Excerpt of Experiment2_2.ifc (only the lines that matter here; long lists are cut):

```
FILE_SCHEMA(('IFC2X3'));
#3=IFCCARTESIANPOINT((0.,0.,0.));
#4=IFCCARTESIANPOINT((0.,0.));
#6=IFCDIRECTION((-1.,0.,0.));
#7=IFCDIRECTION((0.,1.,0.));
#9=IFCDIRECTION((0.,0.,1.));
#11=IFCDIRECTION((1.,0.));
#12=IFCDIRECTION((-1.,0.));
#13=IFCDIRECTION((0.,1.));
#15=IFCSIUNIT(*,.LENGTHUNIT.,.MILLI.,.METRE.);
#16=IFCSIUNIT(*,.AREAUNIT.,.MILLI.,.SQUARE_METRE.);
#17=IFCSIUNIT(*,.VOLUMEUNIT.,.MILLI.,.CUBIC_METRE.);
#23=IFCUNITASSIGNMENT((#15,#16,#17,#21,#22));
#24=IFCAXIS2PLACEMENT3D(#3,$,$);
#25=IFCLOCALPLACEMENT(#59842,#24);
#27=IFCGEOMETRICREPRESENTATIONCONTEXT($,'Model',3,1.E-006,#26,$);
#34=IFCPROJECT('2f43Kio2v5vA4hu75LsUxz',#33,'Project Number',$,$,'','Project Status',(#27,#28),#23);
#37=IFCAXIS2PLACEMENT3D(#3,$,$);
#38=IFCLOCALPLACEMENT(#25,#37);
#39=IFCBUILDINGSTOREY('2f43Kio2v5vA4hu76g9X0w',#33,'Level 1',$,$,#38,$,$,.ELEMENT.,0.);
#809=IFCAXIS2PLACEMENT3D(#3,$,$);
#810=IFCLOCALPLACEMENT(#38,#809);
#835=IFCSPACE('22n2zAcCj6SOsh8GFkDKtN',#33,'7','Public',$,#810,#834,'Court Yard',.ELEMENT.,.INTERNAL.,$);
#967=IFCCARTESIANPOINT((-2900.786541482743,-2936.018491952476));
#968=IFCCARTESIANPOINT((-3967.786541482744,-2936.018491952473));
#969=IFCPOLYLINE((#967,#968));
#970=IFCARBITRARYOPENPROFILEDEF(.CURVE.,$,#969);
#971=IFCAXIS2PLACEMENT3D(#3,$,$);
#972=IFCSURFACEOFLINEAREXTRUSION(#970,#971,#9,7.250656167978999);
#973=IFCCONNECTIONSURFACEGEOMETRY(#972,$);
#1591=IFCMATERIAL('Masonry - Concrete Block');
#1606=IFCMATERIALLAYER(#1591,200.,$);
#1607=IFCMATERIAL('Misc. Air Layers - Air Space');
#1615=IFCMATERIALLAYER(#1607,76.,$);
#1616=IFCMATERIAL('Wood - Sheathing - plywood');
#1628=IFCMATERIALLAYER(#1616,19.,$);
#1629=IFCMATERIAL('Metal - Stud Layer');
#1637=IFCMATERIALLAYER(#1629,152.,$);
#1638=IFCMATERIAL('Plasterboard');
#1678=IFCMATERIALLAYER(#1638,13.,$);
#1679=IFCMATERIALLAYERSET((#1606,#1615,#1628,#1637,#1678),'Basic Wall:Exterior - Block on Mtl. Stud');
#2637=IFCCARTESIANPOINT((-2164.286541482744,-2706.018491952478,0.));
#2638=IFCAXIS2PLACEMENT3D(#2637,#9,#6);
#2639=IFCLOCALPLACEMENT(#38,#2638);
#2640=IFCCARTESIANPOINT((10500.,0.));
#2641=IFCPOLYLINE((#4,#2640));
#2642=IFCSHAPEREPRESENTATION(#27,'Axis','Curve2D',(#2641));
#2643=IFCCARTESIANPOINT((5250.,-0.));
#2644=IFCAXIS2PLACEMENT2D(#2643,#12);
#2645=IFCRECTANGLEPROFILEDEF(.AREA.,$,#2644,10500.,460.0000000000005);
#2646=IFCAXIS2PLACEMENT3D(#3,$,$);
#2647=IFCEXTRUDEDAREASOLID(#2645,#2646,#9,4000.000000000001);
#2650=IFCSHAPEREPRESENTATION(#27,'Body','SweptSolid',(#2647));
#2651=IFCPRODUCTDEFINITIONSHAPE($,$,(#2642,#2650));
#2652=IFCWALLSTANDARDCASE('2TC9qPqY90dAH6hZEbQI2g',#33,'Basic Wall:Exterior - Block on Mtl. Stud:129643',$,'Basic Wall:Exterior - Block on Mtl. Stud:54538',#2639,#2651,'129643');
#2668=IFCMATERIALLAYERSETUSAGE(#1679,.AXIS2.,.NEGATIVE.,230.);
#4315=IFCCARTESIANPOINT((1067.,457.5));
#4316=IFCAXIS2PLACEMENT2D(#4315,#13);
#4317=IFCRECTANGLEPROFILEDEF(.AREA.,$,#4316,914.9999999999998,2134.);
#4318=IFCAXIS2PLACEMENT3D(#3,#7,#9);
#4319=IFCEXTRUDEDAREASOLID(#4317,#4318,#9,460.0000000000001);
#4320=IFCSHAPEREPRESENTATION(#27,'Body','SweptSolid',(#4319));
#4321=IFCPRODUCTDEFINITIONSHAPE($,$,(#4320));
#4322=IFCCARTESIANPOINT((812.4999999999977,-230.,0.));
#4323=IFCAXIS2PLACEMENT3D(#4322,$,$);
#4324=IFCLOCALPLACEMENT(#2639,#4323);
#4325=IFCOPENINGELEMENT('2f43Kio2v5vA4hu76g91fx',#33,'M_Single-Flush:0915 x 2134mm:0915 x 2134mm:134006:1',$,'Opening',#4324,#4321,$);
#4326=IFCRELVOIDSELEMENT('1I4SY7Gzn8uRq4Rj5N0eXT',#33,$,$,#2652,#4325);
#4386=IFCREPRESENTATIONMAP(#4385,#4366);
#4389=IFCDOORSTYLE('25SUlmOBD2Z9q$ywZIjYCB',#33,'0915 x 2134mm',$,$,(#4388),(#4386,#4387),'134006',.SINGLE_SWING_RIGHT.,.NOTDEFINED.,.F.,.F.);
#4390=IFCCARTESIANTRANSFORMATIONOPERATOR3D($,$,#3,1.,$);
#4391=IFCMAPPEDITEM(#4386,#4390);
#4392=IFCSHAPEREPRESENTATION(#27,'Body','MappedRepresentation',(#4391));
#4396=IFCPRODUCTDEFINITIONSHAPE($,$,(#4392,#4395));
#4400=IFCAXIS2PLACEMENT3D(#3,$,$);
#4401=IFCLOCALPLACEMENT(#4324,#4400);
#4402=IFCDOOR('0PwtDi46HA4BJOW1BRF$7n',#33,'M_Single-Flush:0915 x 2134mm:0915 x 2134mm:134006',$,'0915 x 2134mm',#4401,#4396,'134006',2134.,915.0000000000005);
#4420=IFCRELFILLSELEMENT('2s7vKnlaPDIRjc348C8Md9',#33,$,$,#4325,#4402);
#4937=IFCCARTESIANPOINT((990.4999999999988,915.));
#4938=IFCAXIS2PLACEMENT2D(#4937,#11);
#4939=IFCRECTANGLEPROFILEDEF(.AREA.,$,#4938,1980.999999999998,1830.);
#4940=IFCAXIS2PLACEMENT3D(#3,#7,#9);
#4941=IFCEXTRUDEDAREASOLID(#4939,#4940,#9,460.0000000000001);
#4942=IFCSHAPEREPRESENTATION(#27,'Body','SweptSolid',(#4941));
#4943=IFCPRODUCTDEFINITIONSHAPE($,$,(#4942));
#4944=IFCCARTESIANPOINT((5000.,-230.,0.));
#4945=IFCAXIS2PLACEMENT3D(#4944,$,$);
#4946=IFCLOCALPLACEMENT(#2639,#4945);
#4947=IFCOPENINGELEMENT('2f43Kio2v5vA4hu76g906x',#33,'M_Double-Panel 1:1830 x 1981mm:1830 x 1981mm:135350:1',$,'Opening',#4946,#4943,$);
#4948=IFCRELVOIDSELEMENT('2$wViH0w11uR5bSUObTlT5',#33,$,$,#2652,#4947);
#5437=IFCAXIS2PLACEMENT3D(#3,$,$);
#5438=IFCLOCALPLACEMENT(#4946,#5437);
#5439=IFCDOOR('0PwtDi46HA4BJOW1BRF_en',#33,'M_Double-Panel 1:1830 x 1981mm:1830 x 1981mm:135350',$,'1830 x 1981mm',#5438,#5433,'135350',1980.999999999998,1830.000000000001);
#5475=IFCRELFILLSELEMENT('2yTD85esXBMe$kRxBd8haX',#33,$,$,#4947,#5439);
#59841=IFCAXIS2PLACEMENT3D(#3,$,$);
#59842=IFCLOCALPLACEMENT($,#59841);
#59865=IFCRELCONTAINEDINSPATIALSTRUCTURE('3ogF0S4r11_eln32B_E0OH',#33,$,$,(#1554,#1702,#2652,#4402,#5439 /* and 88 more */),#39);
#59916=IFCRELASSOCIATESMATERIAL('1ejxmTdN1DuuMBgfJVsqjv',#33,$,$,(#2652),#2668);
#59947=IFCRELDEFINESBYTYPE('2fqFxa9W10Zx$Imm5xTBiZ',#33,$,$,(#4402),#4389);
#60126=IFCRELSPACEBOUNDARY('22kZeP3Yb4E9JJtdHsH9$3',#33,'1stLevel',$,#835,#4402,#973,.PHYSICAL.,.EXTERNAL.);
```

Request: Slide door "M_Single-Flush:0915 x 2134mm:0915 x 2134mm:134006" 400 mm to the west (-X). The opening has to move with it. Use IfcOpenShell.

```python
import numpy as np
import ifcopenshell
import ifcopenshell.api.geometry
import ifcopenshell.util.placement
import ifcopenshell.util.unit

model = ifcopenshell.open("Experiment2_2.ifc")
unit_scale = ifcopenshell.util.unit.calculate_unit_scale(model)

door = model.by_id(4402)
opening = door.FillsVoids[0].RelatingOpeningElement
wall = opening.VoidsElements[0].RelatingBuildingElement

wall_matrix = ifcopenshell.util.placement.get_local_placement(wall.ObjectPlacement)
shift = wall_matrix[:3, 0] * 0.4 / unit_scale
before = ifcopenshell.util.placement.get_local_placement(door.ObjectPlacement)[:3, 3].copy()

# The door is placed relative to its opening, so it follows when the opening moves.
matrix = ifcopenshell.util.placement.get_local_placement(opening.ObjectPlacement)
matrix[:3, 3] += shift
ifcopenshell.api.geometry.edit_object_placement(
    model, product=opening, matrix=matrix, is_si=False, should_transform_children=True
)

# Space boundary surfaces are stored in each space's coordinates; move them too.
for rel in door.ProvidesBoundaries:
    if not rel.ConnectionGeometry:
        continue
    surface = rel.ConnectionGeometry.SurfaceOnRelatingElement
    space_matrix = ifcopenshell.util.placement.get_local_placement(rel.RelatingSpace.ObjectPlacement)
    point = np.array(surface.Position.Location.Coordinates) + space_matrix[:3, :3].T @ shift
    surface.Position = model.createIfcAxis2Placement3D(
        model.createIfcCartesianPoint(point.tolist()), surface.Position.Axis, surface.Position.RefDirection
    )

after = ifcopenshell.util.placement.get_local_placement(door.ObjectPlacement)[:3, 3]
print("door moved by", (after - before).round(3) + 0.0)

model.write("Experiment2_2_rev.ifc")
```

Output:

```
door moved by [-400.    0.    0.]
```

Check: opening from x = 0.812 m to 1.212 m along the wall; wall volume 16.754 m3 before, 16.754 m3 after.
